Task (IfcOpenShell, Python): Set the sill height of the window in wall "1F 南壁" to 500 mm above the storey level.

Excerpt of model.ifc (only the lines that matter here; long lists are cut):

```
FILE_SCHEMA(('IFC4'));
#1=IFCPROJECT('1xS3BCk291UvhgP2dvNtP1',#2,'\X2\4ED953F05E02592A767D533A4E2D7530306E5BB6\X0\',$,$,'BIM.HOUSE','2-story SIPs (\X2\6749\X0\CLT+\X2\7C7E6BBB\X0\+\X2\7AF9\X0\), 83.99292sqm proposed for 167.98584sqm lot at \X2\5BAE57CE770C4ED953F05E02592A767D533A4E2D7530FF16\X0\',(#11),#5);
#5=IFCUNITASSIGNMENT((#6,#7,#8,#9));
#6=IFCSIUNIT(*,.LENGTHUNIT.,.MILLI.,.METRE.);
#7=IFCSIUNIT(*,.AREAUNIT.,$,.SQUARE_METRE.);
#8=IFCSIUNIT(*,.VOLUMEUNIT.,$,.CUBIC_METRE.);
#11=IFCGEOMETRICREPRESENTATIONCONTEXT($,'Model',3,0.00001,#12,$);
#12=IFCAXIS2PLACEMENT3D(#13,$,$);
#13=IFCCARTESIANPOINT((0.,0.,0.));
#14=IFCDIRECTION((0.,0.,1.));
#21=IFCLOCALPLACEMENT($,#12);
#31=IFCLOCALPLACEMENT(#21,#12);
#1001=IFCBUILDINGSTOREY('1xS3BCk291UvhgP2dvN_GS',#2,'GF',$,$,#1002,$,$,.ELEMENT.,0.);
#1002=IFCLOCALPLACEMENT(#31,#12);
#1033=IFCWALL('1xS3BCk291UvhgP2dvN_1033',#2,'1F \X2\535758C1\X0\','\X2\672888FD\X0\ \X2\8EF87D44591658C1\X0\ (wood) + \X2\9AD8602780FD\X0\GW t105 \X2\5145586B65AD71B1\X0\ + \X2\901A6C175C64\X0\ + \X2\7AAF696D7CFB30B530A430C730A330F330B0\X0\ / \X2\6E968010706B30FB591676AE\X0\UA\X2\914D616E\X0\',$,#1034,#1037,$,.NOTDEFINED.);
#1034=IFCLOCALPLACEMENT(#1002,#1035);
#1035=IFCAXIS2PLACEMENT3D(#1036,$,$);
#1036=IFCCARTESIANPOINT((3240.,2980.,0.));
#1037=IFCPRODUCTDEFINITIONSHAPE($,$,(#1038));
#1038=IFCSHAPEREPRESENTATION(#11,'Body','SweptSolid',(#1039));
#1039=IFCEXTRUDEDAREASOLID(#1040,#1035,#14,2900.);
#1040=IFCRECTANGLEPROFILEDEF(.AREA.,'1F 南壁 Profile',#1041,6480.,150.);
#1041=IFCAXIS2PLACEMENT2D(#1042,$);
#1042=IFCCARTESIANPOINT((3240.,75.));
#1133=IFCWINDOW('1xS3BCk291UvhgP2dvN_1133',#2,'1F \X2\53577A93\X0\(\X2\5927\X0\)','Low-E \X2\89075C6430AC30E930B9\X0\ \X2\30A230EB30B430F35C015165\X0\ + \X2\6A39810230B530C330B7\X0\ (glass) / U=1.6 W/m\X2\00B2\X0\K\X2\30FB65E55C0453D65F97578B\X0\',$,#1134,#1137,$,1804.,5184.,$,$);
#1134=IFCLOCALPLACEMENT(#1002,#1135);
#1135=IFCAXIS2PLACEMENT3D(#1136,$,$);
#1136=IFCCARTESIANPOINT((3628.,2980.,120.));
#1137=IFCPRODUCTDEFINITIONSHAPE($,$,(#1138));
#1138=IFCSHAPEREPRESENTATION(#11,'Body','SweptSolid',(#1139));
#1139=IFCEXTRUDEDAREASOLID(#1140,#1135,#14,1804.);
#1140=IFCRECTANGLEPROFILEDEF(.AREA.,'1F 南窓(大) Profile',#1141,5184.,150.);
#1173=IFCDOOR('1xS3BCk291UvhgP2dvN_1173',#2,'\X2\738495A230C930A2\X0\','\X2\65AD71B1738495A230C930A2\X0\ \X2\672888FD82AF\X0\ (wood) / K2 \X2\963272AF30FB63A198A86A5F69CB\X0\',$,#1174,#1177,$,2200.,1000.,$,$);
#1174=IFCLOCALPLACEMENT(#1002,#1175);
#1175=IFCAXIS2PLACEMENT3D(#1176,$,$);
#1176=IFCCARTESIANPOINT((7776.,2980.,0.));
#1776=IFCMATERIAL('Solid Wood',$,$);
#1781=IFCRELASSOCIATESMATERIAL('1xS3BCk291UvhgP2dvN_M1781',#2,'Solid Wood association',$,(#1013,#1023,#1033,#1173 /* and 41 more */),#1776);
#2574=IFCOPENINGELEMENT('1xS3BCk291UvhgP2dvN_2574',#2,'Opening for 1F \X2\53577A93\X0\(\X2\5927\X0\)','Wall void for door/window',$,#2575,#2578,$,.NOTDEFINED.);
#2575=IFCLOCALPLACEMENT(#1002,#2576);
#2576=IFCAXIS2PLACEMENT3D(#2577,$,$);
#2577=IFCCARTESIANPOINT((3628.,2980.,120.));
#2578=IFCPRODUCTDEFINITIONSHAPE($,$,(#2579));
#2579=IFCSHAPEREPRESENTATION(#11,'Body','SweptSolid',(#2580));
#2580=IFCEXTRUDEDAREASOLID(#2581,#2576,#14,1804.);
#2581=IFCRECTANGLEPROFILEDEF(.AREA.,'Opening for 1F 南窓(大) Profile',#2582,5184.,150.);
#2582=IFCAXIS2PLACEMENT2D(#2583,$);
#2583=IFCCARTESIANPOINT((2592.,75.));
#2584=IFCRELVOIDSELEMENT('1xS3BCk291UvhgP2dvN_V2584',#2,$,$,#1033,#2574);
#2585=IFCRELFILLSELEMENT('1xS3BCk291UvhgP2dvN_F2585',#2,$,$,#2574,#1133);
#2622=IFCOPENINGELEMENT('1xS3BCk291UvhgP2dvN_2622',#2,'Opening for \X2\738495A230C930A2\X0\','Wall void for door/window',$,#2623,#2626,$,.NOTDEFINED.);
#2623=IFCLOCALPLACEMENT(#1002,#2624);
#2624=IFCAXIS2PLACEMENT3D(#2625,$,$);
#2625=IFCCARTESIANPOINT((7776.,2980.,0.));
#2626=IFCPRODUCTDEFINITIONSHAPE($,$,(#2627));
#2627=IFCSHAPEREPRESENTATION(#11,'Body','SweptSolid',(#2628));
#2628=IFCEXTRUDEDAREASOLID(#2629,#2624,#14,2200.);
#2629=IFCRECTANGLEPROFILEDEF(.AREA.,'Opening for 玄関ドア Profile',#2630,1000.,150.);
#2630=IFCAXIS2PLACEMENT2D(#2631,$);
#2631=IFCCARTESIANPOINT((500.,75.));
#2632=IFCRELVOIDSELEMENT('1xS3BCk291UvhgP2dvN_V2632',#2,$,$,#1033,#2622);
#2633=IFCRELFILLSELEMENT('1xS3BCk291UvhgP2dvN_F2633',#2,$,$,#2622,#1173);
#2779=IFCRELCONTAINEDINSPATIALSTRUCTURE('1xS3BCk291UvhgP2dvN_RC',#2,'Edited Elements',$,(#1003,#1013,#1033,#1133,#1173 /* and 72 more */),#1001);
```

```python
import numpy as np
import ifcopenshell
import ifcopenshell.api.geometry
import ifcopenshell.geom
import ifcopenshell.util.element
import ifcopenshell.util.placement
import ifcopenshell.util.shape
import ifcopenshell.util.unit

model = ifcopenshell.open("model.ifc")
unit_scale = ifcopenshell.util.unit.calculate_unit_scale(model)

window = model.by_guid("1xS3BCk291UvhgP2dvN_1133")
opening = window.FillsVoids[0].RelatingOpeningElement
storey = ifcopenshell.util.element.get_container(window, ifc_class="IfcBuildingStorey")
level = ifcopenshell.util.placement.get_local_placement(storey.ObjectPlacement)[2, 3]

# The opening's origin need not be at the sill, so measure its lowest point.
shape = ifcopenshell.geom.create_shape(ifcopenshell.geom.settings(), opening)
bottom = ifcopenshell.util.shape.get_shape_bottom_elevation(shape, shape.geometry) / unit_scale
dz = level + 500.0 - bottom

shift = np.array([0.0, 0.0, dz])
# The window is not placed relative to its opening, so move both.
for product in (opening, window):
    matrix = ifcopenshell.util.placement.get_local_placement(product.ObjectPlacement)
    matrix[:3, 3] += shift
    ifcopenshell.api.geometry.edit_object_placement(model, product=product, matrix=matrix, is_si=False)

print(f"moved by {dz * unit_scale:+.3f} m")

model.write("model_edited.ifc")
```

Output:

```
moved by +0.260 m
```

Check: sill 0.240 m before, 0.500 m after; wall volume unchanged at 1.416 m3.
